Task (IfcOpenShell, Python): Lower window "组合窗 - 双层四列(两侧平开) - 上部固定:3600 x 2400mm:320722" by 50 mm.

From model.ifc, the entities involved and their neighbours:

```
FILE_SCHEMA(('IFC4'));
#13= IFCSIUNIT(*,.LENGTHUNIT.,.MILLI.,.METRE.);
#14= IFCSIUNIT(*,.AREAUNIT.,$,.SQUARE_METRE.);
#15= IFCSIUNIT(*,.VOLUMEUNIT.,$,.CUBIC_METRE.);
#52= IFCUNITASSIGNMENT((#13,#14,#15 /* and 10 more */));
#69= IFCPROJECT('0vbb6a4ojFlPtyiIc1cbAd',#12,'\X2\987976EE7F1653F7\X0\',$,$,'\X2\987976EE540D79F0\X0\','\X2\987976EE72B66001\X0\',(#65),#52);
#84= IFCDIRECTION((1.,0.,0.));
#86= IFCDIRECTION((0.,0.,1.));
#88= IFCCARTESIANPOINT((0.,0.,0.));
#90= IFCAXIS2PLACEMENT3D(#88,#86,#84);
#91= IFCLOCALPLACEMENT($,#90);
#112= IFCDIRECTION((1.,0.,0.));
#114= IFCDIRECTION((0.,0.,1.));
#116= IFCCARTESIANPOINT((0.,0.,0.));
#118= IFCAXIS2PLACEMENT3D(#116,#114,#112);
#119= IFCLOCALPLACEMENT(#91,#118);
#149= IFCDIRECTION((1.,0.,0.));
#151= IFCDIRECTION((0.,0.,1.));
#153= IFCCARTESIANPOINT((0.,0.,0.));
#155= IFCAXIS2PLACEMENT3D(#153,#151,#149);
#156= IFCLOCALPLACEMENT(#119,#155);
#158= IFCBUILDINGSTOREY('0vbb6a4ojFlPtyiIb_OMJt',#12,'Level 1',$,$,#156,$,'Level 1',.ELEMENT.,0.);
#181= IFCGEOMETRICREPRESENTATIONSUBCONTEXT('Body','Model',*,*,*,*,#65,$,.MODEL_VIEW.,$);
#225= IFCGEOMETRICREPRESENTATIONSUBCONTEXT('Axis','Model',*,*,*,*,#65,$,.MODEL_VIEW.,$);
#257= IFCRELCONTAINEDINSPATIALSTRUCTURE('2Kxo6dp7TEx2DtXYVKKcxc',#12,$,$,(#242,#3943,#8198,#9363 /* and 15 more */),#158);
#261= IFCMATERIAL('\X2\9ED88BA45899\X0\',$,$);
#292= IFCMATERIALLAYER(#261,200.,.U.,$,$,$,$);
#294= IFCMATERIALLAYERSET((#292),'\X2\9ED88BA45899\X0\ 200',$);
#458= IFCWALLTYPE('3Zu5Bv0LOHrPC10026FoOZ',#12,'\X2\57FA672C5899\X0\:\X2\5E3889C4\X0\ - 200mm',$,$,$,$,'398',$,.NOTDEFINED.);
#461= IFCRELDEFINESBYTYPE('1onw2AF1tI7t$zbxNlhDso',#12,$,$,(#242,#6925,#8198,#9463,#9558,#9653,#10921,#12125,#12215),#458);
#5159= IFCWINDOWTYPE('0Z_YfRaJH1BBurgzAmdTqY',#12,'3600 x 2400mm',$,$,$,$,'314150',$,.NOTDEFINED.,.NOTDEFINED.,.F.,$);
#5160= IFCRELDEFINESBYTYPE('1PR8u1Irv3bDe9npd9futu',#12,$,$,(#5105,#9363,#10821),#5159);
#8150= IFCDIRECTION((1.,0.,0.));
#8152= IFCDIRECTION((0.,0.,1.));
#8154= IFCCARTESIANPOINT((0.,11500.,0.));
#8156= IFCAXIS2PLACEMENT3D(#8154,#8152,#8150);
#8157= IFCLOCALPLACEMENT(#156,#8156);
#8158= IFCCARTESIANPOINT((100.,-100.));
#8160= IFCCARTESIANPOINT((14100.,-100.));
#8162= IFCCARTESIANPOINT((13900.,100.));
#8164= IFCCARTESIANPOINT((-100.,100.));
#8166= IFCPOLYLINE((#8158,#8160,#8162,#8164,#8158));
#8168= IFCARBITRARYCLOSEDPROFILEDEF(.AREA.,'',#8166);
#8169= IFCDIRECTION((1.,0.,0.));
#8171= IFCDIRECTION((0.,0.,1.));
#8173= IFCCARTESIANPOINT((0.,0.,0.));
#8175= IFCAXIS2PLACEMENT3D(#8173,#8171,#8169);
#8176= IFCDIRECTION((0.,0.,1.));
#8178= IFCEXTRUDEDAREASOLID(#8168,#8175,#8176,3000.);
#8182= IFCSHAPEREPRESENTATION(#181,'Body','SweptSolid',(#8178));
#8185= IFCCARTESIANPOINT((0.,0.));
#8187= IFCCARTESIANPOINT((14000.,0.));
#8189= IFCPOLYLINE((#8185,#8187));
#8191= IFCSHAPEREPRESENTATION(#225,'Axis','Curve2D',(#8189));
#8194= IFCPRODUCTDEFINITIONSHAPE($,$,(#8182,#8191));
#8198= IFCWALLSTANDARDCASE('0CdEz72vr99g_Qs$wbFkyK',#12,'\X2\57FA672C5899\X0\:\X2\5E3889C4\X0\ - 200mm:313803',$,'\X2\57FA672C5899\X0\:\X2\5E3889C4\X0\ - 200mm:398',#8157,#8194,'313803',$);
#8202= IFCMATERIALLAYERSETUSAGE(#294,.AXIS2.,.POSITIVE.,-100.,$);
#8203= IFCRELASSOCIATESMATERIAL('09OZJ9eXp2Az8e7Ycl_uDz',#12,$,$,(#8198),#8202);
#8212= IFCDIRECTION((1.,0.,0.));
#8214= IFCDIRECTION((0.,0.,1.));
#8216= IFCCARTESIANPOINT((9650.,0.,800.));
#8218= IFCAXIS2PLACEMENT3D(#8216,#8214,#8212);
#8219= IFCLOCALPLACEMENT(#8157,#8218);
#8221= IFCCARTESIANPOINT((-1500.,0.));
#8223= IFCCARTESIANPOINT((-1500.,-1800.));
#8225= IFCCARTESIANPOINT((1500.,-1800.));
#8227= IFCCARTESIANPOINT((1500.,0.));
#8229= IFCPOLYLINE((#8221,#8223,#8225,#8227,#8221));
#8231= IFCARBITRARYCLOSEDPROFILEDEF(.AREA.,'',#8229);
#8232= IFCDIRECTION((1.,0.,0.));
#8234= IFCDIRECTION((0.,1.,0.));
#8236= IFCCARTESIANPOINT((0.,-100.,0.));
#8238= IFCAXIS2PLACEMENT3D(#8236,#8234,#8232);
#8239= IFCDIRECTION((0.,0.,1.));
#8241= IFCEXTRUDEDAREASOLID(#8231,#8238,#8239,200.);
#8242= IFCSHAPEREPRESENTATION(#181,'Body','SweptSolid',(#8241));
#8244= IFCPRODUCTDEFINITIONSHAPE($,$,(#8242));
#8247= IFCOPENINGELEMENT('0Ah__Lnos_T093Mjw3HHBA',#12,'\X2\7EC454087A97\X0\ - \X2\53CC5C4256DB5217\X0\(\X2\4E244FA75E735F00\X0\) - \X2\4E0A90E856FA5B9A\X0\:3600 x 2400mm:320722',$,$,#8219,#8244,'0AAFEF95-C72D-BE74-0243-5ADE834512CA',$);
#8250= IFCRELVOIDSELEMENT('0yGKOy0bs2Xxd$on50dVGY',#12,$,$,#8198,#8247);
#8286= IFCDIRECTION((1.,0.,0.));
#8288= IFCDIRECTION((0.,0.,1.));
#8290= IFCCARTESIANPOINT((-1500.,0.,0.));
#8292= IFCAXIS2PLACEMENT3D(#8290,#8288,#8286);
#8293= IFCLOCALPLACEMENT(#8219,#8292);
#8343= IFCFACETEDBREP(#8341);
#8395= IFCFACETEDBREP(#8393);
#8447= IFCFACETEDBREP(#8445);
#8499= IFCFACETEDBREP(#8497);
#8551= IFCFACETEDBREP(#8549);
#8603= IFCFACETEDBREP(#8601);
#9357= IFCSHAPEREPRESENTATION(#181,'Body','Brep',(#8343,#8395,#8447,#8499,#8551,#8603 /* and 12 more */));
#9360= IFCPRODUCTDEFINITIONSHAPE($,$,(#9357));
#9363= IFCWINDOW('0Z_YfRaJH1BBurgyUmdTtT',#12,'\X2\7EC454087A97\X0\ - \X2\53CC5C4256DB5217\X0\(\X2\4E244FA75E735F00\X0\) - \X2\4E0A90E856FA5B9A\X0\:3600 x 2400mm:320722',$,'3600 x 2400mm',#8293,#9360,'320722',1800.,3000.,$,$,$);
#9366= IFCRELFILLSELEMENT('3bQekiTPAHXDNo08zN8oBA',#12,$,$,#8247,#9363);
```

```python
import numpy as np
import ifcopenshell
import ifcopenshell.api.geometry
import ifcopenshell.util.placement
import ifcopenshell.util.unit

model = ifcopenshell.open("model.ifc")
unit_scale = ifcopenshell.util.unit.calculate_unit_scale(model)

window = model.by_guid("0Z_YfRaJH1BBurgyUmdTtT")
opening = window.FillsVoids[0].RelatingOpeningElement
dz = -50.0

shift = np.array([0.0, 0.0, dz])
# The window is placed relative to its opening, so it follows when the opening moves.
matrix = ifcopenshell.util.placement.get_local_placement(opening.ObjectPlacement)
matrix[:3, 3] += shift
ifcopenshell.api.geometry.edit_object_placement(
    model, product=opening, matrix=matrix, is_si=False, should_transform_children=True
)

print(f"moved by {dz * unit_scale:+.3f} m")

model.write("model-out.ifc")
```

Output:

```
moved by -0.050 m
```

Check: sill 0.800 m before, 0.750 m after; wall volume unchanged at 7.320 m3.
